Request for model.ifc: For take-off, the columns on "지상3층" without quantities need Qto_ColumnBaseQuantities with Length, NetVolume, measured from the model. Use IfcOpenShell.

First a look at what the model holds.

```python
import ifcopenshell
import ifcopenshell.util.element
import ifcopenshell.util.unit

model = ifcopenshell.open("model.ifc")
print(model.schema)
for unit_type in ("LENGTHUNIT", "AREAUNIT", "VOLUMEUNIT"):
    print(unit_type, ifcopenshell.util.unit.calculate_unit_scale(model, unit_type))
storey = next(s for s in model.by_type("IfcBuildingStorey") if s.Name == "지상3층")
columns = [e for e in ifcopenshell.util.element.get_decomposition(storey) if e.is_a("IfcColumn")]
for e in sorted(columns, key=lambda e: e.id()):
    print(e.id(), e.is_a(), e.Name, list(ifcopenshell.util.element.get_psets(e, qtos_only=True)), sep=" | ")
```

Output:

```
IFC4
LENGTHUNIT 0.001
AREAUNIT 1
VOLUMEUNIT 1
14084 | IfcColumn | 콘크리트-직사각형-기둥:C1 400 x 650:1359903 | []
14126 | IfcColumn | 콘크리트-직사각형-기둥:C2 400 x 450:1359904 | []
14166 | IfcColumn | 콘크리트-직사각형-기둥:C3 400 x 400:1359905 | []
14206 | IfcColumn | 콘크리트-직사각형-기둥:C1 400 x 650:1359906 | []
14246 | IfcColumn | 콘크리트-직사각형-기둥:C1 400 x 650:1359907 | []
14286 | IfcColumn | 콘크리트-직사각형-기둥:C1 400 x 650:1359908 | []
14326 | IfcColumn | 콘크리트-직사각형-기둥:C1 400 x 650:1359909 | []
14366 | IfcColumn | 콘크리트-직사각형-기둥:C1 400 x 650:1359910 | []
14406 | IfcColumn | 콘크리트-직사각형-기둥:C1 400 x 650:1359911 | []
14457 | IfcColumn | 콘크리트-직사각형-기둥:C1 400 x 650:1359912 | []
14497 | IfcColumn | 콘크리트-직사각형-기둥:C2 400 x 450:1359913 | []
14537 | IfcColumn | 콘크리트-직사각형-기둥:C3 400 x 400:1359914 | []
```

```python
import ifcopenshell
import ifcopenshell.api.pset
import ifcopenshell.geom
import ifcopenshell.util.element
import ifcopenshell.util.shape
import ifcopenshell.util.unit

model = ifcopenshell.open("model.ifc")
unit_scale = ifcopenshell.util.unit.calculate_unit_scale(model)
volume_scale = ifcopenshell.util.unit.calculate_unit_scale(model, "VOLUMEUNIT")
settings = ifcopenshell.geom.settings()

storey = next(s for s in model.by_type("IfcBuildingStorey") if s.Name == "지상3층")
columns = [e for e in ifcopenshell.util.element.get_decomposition(storey) if e.is_a("IfcColumn")]

for e in sorted(columns, key=lambda e: e.id()):
    if ifcopenshell.util.element.get_psets(e, qtos_only=True, should_inherit=False):
        continue
    # Geometry comes back in metres, in the element's own axes.
    shape = ifcopenshell.geom.create_shape(settings, e)
    values = {
        "Length": ifcopenshell.util.shape.get_z(shape.geometry) / unit_scale,
        "NetVolume": ifcopenshell.util.shape.get_volume(shape.geometry) / volume_scale,
    }
    qto = ifcopenshell.api.pset.add_qto(model, product=e, name="Qto_ColumnBaseQuantities")
    ifcopenshell.api.pset.edit_qto(model, qto=qto, properties=values)
    print(e.id(), {k: round(v, 3) for k, v in values.items()})

model.write("model_updated.ifc")
```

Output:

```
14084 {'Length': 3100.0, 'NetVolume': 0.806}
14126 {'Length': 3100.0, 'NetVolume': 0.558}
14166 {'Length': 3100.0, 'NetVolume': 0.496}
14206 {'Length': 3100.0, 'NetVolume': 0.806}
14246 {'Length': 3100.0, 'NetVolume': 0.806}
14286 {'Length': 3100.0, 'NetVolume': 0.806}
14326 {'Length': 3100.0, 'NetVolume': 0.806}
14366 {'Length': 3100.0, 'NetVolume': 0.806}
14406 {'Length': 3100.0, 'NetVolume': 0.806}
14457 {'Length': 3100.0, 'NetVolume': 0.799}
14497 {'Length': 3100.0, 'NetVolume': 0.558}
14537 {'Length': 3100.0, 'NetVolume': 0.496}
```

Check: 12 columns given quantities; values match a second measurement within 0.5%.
